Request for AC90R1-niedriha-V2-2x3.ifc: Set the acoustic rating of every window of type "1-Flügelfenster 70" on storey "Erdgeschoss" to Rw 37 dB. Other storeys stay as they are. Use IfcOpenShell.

First a look at what the model holds.

```python
import ifcopenshell
import ifcopenshell.util.element

model = ifcopenshell.open("AC90R1-niedriha-V2-2x3.ifc")
print(model.schema)
storey = next(s for s in model.by_type("IfcBuildingStorey") if s.Name == "Erdgeschoss")
windows = [e for e in ifcopenshell.util.element.get_decomposition(storey) if e.is_a("IfcWindow")]
seen = {}
for e in windows:
    element_type = ifcopenshell.util.element.get_type(e)
    key = (element_type.Name if element_type != e and element_type else None, ifcopenshell.util.element.get_pset(e, "Pset_WindowCommon", "AcousticRating"))
    seen[key] = seen.get(key, 0) + 1
for (name, value), count in sorted(seen.items(), key=str):
    print(count, "x", name, "|", value)
```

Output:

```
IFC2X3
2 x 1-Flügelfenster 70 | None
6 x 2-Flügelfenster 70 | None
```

```python
import ifcopenshell
import ifcopenshell.api.pset
import ifcopenshell.util.element

model = ifcopenshell.open("AC90R1-niedriha-V2-2x3.ifc")

storey = next(s for s in model.by_type("IfcBuildingStorey") if s.Name == "Erdgeschoss")
windows = [e for e in ifcopenshell.util.element.get_decomposition(storey) if e.is_a("IfcWindow")]

count = 0
for e in windows:
    element_type = ifcopenshell.util.element.get_type(e)
    if element_type in (None, e) or element_type.Name != "1-Flügelfenster 70":
        continue
    # add_pset returns the element's existing set when there is one.
    pset = ifcopenshell.api.pset.add_pset(model, product=e, name="Pset_WindowCommon")
    ifcopenshell.api.pset.edit_pset(model, pset=pset, properties={"AcousticRating": "Rw 37 dB"})
    count += 1

print(count, "windows updated")

model.write("AC90R1-niedriha-V2-2x3_edited.ifc")
```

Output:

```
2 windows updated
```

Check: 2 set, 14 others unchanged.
